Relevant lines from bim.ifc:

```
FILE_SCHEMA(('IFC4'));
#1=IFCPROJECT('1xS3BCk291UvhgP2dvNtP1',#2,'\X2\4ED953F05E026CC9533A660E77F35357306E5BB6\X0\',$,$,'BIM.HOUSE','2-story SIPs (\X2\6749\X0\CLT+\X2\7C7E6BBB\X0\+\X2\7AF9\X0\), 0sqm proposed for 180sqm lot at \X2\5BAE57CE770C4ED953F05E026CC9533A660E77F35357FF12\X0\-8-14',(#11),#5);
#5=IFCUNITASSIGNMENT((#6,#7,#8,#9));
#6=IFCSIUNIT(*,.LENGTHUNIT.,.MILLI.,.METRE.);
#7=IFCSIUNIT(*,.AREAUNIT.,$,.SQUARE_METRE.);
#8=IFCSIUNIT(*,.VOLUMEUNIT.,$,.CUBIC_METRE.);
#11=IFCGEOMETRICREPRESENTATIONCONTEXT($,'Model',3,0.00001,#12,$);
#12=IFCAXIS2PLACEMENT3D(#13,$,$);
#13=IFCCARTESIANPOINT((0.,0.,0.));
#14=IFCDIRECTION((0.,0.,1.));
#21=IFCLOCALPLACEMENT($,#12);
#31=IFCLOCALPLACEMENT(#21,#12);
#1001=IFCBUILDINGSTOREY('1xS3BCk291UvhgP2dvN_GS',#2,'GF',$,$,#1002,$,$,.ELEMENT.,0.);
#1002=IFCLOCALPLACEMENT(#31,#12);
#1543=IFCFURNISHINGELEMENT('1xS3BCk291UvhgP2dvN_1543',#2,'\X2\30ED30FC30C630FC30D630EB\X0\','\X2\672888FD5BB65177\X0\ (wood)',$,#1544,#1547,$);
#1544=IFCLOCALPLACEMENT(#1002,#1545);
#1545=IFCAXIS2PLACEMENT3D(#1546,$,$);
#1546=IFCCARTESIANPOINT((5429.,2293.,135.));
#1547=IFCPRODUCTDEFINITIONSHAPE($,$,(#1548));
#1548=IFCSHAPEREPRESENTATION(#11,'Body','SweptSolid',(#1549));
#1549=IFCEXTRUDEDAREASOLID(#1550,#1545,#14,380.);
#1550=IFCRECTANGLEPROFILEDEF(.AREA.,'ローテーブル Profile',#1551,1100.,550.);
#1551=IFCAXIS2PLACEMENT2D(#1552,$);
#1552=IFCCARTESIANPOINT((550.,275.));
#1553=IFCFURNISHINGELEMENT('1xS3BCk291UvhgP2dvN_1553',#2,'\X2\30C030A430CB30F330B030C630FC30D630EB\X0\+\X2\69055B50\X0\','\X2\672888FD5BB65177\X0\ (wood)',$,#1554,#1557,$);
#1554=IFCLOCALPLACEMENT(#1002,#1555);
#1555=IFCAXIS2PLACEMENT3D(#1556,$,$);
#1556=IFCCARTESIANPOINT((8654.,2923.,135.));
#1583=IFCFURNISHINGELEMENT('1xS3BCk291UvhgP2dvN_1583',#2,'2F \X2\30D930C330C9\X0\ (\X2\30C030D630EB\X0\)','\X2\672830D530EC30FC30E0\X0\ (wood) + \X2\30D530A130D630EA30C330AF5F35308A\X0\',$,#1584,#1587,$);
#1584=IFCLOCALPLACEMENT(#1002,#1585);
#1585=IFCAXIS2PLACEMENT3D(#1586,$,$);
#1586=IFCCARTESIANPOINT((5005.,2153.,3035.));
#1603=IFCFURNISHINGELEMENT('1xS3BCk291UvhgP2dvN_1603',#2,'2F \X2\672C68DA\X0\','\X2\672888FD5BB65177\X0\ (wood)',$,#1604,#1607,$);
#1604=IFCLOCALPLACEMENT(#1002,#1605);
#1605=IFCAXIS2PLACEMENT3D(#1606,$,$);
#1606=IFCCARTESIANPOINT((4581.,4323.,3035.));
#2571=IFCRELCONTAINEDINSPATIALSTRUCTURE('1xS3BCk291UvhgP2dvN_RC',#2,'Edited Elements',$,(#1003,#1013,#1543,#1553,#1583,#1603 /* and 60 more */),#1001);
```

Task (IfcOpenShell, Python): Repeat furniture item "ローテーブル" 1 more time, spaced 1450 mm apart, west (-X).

```python
import numpy as np
import ifcopenshell
import ifcopenshell.api.geometry
import ifcopenshell.api.root
import ifcopenshell.util.element
import ifcopenshell.util.placement

model = ifcopenshell.open("bim.ifc")


def reuse_history(source, copy):
    """copy_class also copies each property set's owner history, people and application; keep the originals."""
    for rel in copy.IsDefinedBy:
        if rel.is_a("IfcRelDefinesByProperties") and (history := rel.RelatingPropertyDefinition.OwnerHistory):
            rel.RelatingPropertyDefinition.OwnerHistory = source.OwnerHistory
            ifcopenshell.util.element.remove_deep2(model, history)


source = model.by_guid("1xS3BCk291UvhgP2dvN_1543")
base = ifcopenshell.util.placement.get_local_placement(source.ObjectPlacement)
step = np.array([-1.0, 0.0, 0.0]) * 1450.0

for i in range(1, 2):
    copy = ifcopenshell.api.root.copy_class(model, product=source)
    copy.Representation = ifcopenshell.util.element.copy_deep(
        model, source.Representation, exclude=["IfcGeometricRepresentationContext", "IfcRepresentationMap"]
    )
    reuse_history(source, copy)
    matrix = base.copy()
    matrix[:3, 3] += i * step
    print("added at", matrix[:3, 3].round(3) + 0.0)
    ifcopenshell.api.geometry.edit_object_placement(model, product=copy, matrix=matrix, is_si=False)

model.write("bim_rev.ifc")
```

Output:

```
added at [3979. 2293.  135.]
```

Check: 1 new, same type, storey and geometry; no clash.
